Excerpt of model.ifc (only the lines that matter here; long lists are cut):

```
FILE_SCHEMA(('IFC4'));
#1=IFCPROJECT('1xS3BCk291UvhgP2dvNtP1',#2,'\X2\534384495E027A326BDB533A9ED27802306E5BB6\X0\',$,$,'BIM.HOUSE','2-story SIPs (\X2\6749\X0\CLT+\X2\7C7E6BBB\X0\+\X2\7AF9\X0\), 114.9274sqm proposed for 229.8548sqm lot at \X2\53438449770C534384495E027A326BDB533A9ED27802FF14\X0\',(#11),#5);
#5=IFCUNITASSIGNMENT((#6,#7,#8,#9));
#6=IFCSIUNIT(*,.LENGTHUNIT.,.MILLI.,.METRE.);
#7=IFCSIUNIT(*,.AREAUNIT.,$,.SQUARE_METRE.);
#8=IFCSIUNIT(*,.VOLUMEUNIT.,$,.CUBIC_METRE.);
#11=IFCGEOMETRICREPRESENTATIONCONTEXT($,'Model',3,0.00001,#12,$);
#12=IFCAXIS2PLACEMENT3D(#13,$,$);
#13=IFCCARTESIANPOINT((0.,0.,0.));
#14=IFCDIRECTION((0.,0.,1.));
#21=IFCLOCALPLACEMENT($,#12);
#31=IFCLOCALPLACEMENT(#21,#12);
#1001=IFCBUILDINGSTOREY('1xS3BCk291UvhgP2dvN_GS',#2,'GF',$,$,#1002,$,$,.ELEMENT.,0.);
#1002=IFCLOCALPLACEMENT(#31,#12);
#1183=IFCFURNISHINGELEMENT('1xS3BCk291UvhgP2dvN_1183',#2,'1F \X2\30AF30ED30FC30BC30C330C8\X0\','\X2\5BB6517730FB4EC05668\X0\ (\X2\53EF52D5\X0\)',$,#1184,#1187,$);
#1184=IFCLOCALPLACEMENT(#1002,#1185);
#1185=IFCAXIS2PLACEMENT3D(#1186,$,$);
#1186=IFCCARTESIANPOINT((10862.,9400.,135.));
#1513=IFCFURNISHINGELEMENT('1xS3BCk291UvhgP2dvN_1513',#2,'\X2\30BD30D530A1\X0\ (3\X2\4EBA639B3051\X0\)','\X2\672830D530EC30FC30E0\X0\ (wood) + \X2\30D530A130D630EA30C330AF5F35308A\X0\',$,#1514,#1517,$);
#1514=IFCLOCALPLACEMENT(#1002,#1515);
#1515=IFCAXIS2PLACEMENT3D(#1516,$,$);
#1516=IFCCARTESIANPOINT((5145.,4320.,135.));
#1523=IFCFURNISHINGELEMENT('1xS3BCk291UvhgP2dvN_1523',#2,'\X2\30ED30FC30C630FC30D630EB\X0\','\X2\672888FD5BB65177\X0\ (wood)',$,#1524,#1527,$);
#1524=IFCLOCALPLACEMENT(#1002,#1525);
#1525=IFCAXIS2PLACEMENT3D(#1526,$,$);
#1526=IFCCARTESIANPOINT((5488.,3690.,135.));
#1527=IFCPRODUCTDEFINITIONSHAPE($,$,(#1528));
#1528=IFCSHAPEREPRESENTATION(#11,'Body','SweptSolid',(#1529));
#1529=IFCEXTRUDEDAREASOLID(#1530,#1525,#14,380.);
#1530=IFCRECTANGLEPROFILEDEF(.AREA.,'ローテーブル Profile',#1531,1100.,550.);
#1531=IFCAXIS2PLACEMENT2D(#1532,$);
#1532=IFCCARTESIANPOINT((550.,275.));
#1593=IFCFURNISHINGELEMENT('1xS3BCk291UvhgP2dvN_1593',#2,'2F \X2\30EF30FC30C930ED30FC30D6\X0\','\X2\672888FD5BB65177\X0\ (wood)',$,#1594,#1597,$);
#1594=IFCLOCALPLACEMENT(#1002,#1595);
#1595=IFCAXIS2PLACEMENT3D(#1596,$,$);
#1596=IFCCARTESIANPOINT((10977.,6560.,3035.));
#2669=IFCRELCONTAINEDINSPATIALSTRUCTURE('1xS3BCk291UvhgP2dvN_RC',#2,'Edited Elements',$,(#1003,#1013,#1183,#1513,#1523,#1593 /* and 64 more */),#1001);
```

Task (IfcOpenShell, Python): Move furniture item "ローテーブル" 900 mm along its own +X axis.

```python
import ifcopenshell
import ifcopenshell.api.geometry
import ifcopenshell.util.placement

model = ifcopenshell.open("model.ifc")

item = model.by_guid("1xS3BCk291UvhgP2dvN_1523")
matrix = ifcopenshell.util.placement.get_local_placement(item.ObjectPlacement)
matrix[:3, 3] += matrix[:3, 0] * 900.0
ifcopenshell.api.geometry.edit_object_placement(model, product=item, matrix=matrix, is_si=False)

print(ifcopenshell.util.placement.get_local_placement(item.ObjectPlacement).round(3) + 0.0)

model.write("model_v2.ifc")
```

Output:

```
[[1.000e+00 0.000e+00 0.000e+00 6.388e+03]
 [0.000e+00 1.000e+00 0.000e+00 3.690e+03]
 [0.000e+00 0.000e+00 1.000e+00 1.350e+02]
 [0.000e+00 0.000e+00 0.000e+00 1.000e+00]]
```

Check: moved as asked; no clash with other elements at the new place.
